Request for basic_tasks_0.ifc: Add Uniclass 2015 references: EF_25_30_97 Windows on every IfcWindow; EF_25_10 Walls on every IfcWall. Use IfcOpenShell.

First a look at what the model holds.

```python
import ifcopenshell

model = ifcopenshell.open("basic_tasks_0.ifc")
print(model.schema)
print("classifications:", [c.Name for c in model.by_type("IfcClassification")])
for ifc_class in ("IfcDoor", "IfcRoof", "IfcStair", "IfcWall", "IfcWindow"):
    print(ifc_class, len(model.by_type(ifc_class)))
```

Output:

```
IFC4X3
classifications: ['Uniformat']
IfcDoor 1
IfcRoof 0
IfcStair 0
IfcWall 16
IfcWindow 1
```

```python
import ifcopenshell
import ifcopenshell.api.classification

model = ifcopenshell.open("basic_tasks_0.ifc")

system = ifcopenshell.api.classification.add_classification(model, classification="Uniclass 2015")

codes = {
    "IfcWindow": ("EF_25_30_97", "Windows"),
    "IfcWall": ("EF_25_10", "Walls"),
}
for ifc_class, (code, name) in codes.items():
    products = model.by_type(ifc_class)
    ifcopenshell.api.classification.add_reference(
        model, products=products, classification=system, identification=code, name=name
    )
    print(code, len(products))

model.write("basic_tasks_0_edited.ifc")
```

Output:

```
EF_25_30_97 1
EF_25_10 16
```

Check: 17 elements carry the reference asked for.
